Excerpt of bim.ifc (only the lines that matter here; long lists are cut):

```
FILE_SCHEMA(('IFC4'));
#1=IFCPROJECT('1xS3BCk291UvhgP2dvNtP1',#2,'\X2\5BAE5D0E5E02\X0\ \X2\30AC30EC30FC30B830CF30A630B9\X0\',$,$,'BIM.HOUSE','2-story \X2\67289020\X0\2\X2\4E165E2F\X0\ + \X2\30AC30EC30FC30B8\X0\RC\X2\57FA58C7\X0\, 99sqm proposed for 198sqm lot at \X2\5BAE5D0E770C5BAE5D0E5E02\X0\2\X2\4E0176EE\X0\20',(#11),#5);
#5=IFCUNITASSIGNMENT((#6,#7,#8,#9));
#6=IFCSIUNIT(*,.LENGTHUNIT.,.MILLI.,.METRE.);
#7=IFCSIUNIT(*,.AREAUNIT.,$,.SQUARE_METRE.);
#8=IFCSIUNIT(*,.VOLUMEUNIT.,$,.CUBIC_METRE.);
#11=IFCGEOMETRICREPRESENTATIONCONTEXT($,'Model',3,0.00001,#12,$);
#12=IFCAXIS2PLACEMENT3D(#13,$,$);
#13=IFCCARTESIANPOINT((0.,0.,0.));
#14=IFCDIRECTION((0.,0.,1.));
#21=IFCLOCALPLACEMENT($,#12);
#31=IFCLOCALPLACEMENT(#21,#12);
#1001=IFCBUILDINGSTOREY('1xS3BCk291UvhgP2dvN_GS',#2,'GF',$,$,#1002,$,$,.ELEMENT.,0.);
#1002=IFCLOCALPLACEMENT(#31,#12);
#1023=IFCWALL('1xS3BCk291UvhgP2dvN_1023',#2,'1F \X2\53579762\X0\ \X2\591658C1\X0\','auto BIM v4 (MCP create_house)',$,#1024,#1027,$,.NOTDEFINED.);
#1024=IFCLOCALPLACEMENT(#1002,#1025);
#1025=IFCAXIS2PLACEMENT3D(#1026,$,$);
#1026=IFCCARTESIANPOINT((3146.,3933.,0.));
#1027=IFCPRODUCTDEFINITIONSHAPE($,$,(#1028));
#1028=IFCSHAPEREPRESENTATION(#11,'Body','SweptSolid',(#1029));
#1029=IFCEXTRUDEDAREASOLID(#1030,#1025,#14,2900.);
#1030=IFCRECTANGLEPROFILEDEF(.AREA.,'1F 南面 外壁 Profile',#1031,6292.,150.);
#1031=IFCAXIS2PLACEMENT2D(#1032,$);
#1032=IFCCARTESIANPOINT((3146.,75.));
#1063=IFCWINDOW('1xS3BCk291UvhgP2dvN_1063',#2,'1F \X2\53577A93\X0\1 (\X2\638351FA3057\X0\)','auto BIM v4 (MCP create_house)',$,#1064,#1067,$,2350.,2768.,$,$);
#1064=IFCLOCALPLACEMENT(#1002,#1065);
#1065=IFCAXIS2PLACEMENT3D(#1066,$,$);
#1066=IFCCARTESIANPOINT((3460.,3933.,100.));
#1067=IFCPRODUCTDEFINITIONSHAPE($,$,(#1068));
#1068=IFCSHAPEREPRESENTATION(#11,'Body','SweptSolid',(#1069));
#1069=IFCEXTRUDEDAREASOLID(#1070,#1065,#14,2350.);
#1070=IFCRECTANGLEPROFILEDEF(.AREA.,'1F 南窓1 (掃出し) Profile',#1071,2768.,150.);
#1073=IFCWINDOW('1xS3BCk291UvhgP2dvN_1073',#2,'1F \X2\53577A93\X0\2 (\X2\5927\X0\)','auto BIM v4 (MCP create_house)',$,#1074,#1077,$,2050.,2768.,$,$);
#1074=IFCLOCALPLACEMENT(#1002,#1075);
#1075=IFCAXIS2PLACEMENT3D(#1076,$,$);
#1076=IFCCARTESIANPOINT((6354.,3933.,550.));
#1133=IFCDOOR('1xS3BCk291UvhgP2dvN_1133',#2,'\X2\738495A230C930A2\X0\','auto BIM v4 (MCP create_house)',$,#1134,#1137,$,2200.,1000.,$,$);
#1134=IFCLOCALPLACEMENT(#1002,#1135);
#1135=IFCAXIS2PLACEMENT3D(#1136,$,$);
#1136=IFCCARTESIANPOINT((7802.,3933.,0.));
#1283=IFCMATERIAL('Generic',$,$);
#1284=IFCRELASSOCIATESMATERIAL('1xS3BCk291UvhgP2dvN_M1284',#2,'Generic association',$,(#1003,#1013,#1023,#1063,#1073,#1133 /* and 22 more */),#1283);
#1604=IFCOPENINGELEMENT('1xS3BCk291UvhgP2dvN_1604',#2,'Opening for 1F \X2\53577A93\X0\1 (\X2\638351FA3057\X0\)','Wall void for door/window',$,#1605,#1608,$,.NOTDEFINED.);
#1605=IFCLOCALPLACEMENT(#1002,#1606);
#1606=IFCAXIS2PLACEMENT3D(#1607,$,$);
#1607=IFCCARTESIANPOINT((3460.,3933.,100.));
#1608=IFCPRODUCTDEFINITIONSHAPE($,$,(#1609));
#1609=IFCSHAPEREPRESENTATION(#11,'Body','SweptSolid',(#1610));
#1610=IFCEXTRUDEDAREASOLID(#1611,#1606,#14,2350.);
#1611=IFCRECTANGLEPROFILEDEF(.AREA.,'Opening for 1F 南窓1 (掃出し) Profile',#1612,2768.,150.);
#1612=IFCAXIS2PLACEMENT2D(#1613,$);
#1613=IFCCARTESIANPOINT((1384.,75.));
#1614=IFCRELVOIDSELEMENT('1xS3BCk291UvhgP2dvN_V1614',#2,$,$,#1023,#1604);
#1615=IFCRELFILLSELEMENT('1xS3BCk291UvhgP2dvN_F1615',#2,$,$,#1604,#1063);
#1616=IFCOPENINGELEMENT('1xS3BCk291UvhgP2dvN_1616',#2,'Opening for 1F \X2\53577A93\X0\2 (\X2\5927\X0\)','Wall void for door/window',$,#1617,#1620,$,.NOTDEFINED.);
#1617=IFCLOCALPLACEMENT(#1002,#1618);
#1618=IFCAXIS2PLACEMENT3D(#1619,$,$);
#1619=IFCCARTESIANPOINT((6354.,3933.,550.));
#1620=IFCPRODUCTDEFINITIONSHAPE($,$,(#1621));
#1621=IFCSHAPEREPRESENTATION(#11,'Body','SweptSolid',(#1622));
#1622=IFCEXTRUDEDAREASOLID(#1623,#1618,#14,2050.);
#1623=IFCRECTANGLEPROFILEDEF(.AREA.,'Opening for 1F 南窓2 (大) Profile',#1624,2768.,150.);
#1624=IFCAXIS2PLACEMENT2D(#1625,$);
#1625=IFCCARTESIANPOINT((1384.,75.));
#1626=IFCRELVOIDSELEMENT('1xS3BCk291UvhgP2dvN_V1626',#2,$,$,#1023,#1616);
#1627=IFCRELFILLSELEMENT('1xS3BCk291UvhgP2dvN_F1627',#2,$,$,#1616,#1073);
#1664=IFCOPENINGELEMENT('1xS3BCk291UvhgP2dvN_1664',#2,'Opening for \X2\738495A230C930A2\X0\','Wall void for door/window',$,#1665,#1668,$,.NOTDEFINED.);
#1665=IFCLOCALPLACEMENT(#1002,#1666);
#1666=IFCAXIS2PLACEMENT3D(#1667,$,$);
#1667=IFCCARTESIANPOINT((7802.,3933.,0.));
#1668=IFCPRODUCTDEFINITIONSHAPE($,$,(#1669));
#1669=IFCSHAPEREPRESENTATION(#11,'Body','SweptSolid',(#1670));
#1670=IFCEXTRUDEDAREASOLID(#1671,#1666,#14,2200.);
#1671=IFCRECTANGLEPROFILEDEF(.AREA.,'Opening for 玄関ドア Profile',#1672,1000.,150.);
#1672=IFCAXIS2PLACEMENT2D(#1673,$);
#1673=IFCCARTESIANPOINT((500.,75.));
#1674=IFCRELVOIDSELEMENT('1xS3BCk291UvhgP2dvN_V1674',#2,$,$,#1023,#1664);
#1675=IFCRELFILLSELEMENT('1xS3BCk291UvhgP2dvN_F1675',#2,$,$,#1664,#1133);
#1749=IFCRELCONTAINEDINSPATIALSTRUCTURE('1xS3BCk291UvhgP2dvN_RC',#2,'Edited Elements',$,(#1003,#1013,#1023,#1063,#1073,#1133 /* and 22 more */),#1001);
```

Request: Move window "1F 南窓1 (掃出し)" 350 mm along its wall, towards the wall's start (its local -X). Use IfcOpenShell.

```python
import ifcopenshell
import ifcopenshell.api.geometry
import ifcopenshell.util.placement
import ifcopenshell.util.unit

model = ifcopenshell.open("bim.ifc")
unit_scale = ifcopenshell.util.unit.calculate_unit_scale(model)

window = model.by_guid("1xS3BCk291UvhgP2dvN_1063")
opening = window.FillsVoids[0].RelatingOpeningElement
wall = opening.VoidsElements[0].RelatingBuildingElement

wall_matrix = ifcopenshell.util.placement.get_local_placement(wall.ObjectPlacement)
shift = wall_matrix[:3, 0] * -0.35 / unit_scale
before = ifcopenshell.util.placement.get_local_placement(window.ObjectPlacement)[:3, 3].copy()

# The window is not placed relative to its opening, so move both.
for product in (opening, window):
    matrix = ifcopenshell.util.placement.get_local_placement(product.ObjectPlacement)
    matrix[:3, 3] += shift
    ifcopenshell.api.geometry.edit_object_placement(model, product=product, matrix=matrix, is_si=False)

after = ifcopenshell.util.placement.get_local_placement(window.ObjectPlacement)[:3, 3]
print("window moved by", (after - before).round(3) + 0.0)

model.write("bim_edited.ifc")
```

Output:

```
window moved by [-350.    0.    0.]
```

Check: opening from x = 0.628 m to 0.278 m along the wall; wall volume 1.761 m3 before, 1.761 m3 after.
